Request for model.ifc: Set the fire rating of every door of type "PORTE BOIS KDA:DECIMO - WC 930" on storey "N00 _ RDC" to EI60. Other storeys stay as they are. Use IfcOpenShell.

First a look at what the model holds.

```python
import ifcopenshell
import ifcopenshell.util.element

model = ifcopenshell.open("model.ifc")
print(model.schema)
storey = next(s for s in model.by_type("IfcBuildingStorey") if s.Name == "N00 _ RDC")
doors = [e for e in ifcopenshell.util.element.get_decomposition(storey) if e.is_a("IfcDoor")]
seen = {}
for e in doors:
    element_type = ifcopenshell.util.element.get_type(e)
    key = (element_type.Name if element_type != e and element_type else None, ifcopenshell.util.element.get_pset(e, "Pset_DoorCommon", "FireRating"))
    seen[key] = seen.get(key, 0) + 1
for (name, value), count in sorted(seen.items(), key=str):
    print(count, "x", name, "|", value)
```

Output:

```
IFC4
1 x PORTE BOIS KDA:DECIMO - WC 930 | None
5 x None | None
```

```python
import ifcopenshell
import ifcopenshell.api.pset
import ifcopenshell.util.element

model = ifcopenshell.open("model.ifc")

storey = next(s for s in model.by_type("IfcBuildingStorey") if s.Name == "N00 _ RDC")
doors = [e for e in ifcopenshell.util.element.get_decomposition(storey) if e.is_a("IfcDoor")]

count = 0
for e in doors:
    element_type = ifcopenshell.util.element.get_type(e)
    if element_type in (None, e) or element_type.Name != "PORTE BOIS KDA:DECIMO - WC 930":
        continue
    # add_pset returns the element's existing set when there is one.
    pset = ifcopenshell.api.pset.add_pset(model, product=e, name="Pset_DoorCommon")
    ifcopenshell.api.pset.edit_pset(model, pset=pset, properties={"FireRating": "EI60"})
    count += 1

print(count, "doors updated")

model.write("model_rev.ifc")
```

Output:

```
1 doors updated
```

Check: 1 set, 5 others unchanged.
